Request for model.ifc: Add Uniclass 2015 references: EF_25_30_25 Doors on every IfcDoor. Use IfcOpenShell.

First a look at what the model holds.

```python
import ifcopenshell

model = ifcopenshell.open("model.ifc")
print(model.schema)
print("classifications:", [c.Name for c in model.by_type("IfcClassification")])
for ifc_class in ("IfcDoor", "IfcRoof", "IfcStair", "IfcWall", "IfcWindow"):
    print(ifc_class, len(model.by_type(ifc_class)))
```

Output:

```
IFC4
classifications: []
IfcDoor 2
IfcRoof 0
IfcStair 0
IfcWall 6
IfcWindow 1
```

```python
import ifcopenshell
import ifcopenshell.api.classification

model = ifcopenshell.open("model.ifc")

system = ifcopenshell.api.classification.add_classification(model, classification="Uniclass 2015")

codes = {
    "IfcDoor": ("EF_25_30_25", "Doors"),
}
for ifc_class, (code, name) in codes.items():
    products = model.by_type(ifc_class)
    ifcopenshell.api.classification.add_reference(
        model, products=products, classification=system, identification=code, name=name
    )
    print(code, len(products))

model.write("model_edited.ifc")
```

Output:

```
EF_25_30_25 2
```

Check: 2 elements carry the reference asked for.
